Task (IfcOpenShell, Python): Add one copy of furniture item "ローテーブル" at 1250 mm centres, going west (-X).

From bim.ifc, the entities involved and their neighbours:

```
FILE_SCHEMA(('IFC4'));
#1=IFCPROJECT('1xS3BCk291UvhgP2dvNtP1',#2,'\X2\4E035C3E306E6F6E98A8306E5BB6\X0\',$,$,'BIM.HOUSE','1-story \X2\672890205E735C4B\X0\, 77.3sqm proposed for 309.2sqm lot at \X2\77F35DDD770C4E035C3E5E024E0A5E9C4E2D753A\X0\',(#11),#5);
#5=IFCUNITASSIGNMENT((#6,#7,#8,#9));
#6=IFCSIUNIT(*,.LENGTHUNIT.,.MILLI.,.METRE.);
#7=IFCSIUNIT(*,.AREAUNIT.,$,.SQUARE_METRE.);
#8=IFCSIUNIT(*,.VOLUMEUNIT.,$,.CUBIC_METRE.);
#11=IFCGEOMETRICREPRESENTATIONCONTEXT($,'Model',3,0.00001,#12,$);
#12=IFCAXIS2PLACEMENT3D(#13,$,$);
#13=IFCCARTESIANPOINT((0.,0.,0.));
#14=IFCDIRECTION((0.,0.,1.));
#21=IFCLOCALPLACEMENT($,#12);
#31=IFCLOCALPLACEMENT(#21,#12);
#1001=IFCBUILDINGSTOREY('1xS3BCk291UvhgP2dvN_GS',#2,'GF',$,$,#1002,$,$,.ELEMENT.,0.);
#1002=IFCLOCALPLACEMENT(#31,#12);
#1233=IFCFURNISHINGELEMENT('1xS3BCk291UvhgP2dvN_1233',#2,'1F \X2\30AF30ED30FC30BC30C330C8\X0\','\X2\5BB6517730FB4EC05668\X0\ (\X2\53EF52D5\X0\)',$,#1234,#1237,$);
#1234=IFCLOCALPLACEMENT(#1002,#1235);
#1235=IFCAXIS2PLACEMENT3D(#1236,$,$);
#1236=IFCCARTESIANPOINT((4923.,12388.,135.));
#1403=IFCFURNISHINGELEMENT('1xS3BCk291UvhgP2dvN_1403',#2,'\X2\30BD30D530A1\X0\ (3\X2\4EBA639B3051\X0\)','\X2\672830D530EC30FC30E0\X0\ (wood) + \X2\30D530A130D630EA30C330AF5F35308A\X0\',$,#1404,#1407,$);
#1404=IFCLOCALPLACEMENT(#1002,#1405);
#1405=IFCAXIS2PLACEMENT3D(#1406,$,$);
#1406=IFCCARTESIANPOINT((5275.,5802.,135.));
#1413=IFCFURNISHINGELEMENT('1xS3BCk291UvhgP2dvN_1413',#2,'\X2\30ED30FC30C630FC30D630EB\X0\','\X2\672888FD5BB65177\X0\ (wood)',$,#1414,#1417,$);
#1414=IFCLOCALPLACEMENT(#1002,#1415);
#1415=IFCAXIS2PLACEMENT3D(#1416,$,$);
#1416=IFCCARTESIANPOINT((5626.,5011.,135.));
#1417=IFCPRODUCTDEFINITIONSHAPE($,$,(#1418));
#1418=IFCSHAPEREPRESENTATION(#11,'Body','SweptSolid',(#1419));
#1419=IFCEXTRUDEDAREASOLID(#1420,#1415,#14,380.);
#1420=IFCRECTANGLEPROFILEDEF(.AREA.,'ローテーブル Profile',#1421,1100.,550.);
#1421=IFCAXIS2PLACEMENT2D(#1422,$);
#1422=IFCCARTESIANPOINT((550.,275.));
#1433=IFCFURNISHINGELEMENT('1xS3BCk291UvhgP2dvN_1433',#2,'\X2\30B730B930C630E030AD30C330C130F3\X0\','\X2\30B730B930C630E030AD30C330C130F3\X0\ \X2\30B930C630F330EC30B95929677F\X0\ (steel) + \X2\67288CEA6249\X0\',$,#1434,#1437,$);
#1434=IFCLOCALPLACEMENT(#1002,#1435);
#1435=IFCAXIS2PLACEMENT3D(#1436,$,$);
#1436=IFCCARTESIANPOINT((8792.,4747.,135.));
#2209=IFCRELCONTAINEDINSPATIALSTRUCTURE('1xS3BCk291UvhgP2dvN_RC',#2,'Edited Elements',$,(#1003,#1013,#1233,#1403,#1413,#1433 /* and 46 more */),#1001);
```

```python
import numpy as np
import ifcopenshell
import ifcopenshell.api.geometry
import ifcopenshell.api.root
import ifcopenshell.util.element
import ifcopenshell.util.placement

model = ifcopenshell.open("bim.ifc")


def reuse_history(source, copy):
    """copy_class also copies each property set's owner history, people and application; keep the originals."""
    for rel in copy.IsDefinedBy:
        if rel.is_a("IfcRelDefinesByProperties") and (history := rel.RelatingPropertyDefinition.OwnerHistory):
            rel.RelatingPropertyDefinition.OwnerHistory = source.OwnerHistory
            ifcopenshell.util.element.remove_deep2(model, history)


source = model.by_guid("1xS3BCk291UvhgP2dvN_1413")
base = ifcopenshell.util.placement.get_local_placement(source.ObjectPlacement)
step = np.array([-1.0, 0.0, 0.0]) * 1250.0

for i in range(1, 2):
    copy = ifcopenshell.api.root.copy_class(model, product=source)
    copy.Representation = ifcopenshell.util.element.copy_deep(
        model, source.Representation, exclude=["IfcGeometricRepresentationContext", "IfcRepresentationMap"]
    )
    reuse_history(source, copy)
    matrix = base.copy()
    matrix[:3, 3] += i * step
    print("added at", matrix[:3, 3].round(3) + 0.0)
    ifcopenshell.api.geometry.edit_object_placement(model, product=copy, matrix=matrix, is_si=False)

model.write("bim-out.ifc")
```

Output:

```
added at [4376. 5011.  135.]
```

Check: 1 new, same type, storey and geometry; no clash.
